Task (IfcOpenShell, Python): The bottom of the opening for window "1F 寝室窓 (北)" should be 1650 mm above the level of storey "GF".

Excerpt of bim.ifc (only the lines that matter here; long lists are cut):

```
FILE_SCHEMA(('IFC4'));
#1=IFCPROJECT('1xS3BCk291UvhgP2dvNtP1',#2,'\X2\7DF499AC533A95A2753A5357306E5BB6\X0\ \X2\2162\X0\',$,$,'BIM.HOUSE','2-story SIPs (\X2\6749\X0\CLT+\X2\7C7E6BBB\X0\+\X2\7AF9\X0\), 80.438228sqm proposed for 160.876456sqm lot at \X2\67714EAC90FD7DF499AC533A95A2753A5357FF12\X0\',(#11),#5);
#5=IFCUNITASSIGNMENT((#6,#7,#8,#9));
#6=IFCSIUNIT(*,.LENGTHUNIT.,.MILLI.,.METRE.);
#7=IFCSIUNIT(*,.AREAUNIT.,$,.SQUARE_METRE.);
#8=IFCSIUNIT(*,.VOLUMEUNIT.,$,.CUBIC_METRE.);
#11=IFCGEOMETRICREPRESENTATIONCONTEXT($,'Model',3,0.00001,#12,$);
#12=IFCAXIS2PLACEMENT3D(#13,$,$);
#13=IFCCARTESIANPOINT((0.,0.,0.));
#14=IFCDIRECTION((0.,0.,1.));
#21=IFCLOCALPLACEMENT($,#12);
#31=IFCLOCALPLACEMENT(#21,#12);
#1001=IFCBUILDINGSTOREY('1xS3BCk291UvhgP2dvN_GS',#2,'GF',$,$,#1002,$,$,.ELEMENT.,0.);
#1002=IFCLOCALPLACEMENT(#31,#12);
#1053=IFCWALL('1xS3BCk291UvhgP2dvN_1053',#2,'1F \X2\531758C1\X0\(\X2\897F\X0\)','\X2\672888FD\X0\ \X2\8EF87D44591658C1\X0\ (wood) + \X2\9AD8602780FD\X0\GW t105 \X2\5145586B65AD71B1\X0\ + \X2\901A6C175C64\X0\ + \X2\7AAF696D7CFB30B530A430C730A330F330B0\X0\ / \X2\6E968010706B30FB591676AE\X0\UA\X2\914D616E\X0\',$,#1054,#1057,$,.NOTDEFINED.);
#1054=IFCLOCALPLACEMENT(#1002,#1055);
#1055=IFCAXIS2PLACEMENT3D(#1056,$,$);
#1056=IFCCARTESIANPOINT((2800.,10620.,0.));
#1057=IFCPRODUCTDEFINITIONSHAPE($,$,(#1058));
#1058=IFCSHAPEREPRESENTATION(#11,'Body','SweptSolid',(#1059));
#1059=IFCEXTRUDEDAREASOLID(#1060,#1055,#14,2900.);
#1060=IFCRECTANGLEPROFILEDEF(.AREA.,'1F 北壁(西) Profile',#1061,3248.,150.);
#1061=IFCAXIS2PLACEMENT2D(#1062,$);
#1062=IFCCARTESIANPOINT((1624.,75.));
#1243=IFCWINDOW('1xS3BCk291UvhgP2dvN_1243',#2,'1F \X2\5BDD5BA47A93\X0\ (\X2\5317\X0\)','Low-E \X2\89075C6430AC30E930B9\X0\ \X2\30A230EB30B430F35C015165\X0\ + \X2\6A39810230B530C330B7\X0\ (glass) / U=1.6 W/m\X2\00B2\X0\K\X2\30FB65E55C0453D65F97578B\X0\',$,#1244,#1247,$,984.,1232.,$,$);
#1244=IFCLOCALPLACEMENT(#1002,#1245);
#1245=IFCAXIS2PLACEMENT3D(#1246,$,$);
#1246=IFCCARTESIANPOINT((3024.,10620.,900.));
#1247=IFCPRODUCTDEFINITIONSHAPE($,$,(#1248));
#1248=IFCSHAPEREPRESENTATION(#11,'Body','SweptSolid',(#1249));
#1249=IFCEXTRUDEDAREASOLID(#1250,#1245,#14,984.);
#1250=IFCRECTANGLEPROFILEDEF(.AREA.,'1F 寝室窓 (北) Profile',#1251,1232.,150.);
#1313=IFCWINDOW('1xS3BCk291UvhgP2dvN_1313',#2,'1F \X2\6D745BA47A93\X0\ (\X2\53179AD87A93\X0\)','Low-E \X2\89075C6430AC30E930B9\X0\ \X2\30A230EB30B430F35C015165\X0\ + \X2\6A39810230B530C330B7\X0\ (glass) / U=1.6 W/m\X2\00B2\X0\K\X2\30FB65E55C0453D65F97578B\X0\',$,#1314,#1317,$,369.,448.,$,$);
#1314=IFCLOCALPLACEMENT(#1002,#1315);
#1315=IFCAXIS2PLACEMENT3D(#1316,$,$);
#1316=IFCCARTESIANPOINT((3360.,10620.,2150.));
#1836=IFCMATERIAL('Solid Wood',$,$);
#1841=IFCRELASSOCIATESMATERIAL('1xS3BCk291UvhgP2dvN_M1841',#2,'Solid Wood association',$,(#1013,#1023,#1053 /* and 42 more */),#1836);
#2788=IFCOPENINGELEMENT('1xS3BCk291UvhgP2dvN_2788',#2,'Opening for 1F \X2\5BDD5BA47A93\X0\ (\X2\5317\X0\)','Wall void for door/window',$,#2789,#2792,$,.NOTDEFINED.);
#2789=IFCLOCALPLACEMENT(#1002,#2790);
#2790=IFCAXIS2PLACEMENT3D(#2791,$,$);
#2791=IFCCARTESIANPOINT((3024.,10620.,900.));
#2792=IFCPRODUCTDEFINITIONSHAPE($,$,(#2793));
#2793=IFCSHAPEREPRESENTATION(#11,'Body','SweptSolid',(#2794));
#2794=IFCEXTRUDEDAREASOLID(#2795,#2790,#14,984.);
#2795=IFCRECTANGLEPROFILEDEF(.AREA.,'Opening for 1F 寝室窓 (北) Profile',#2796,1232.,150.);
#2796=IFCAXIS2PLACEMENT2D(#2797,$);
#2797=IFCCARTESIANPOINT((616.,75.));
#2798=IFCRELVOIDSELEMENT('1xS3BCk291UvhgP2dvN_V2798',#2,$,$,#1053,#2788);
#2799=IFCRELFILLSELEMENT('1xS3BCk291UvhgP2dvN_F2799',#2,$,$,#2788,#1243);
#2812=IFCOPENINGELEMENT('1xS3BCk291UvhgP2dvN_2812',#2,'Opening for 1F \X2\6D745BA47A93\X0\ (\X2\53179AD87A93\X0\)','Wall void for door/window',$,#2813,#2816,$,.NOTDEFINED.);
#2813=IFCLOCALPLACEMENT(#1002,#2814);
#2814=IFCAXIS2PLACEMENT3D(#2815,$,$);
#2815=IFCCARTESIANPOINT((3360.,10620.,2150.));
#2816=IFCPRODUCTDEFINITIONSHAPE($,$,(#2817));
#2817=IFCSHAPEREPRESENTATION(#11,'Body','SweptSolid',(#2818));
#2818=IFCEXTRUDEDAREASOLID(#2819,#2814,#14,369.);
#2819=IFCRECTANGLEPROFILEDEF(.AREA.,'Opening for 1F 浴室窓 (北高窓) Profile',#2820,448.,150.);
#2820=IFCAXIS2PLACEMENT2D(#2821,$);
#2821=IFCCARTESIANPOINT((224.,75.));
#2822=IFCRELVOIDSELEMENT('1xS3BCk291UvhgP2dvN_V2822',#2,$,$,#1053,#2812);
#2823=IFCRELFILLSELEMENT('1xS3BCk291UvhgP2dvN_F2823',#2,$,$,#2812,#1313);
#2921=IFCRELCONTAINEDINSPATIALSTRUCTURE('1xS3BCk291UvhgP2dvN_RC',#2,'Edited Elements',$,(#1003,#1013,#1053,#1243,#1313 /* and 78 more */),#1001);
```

```python
import numpy as np
import ifcopenshell
import ifcopenshell.api.geometry
import ifcopenshell.geom
import ifcopenshell.util.element
import ifcopenshell.util.placement
import ifcopenshell.util.shape
import ifcopenshell.util.unit

model = ifcopenshell.open("bim.ifc")
unit_scale = ifcopenshell.util.unit.calculate_unit_scale(model)

window = model.by_guid("1xS3BCk291UvhgP2dvN_1243")
opening = window.FillsVoids[0].RelatingOpeningElement
storey = ifcopenshell.util.element.get_container(window, ifc_class="IfcBuildingStorey")
level = ifcopenshell.util.placement.get_local_placement(storey.ObjectPlacement)[2, 3]

# The opening's origin need not be at the sill, so measure its lowest point.
shape = ifcopenshell.geom.create_shape(ifcopenshell.geom.settings(), opening)
bottom = ifcopenshell.util.shape.get_shape_bottom_elevation(shape, shape.geometry) / unit_scale
dz = level + 1.65 / unit_scale - bottom

shift = np.array([0.0, 0.0, dz])
# The window is not placed relative to its opening, so move both.
for product in (opening, window):
    matrix = ifcopenshell.util.placement.get_local_placement(product.ObjectPlacement)
    matrix[:3, 3] += shift
    ifcopenshell.api.geometry.edit_object_placement(model, product=product, matrix=matrix, is_si=False)

print(f"moved by {dz * unit_scale:+.3f} m")

model.write("bim-out.ifc")
```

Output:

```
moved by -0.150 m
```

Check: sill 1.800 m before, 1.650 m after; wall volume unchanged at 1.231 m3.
